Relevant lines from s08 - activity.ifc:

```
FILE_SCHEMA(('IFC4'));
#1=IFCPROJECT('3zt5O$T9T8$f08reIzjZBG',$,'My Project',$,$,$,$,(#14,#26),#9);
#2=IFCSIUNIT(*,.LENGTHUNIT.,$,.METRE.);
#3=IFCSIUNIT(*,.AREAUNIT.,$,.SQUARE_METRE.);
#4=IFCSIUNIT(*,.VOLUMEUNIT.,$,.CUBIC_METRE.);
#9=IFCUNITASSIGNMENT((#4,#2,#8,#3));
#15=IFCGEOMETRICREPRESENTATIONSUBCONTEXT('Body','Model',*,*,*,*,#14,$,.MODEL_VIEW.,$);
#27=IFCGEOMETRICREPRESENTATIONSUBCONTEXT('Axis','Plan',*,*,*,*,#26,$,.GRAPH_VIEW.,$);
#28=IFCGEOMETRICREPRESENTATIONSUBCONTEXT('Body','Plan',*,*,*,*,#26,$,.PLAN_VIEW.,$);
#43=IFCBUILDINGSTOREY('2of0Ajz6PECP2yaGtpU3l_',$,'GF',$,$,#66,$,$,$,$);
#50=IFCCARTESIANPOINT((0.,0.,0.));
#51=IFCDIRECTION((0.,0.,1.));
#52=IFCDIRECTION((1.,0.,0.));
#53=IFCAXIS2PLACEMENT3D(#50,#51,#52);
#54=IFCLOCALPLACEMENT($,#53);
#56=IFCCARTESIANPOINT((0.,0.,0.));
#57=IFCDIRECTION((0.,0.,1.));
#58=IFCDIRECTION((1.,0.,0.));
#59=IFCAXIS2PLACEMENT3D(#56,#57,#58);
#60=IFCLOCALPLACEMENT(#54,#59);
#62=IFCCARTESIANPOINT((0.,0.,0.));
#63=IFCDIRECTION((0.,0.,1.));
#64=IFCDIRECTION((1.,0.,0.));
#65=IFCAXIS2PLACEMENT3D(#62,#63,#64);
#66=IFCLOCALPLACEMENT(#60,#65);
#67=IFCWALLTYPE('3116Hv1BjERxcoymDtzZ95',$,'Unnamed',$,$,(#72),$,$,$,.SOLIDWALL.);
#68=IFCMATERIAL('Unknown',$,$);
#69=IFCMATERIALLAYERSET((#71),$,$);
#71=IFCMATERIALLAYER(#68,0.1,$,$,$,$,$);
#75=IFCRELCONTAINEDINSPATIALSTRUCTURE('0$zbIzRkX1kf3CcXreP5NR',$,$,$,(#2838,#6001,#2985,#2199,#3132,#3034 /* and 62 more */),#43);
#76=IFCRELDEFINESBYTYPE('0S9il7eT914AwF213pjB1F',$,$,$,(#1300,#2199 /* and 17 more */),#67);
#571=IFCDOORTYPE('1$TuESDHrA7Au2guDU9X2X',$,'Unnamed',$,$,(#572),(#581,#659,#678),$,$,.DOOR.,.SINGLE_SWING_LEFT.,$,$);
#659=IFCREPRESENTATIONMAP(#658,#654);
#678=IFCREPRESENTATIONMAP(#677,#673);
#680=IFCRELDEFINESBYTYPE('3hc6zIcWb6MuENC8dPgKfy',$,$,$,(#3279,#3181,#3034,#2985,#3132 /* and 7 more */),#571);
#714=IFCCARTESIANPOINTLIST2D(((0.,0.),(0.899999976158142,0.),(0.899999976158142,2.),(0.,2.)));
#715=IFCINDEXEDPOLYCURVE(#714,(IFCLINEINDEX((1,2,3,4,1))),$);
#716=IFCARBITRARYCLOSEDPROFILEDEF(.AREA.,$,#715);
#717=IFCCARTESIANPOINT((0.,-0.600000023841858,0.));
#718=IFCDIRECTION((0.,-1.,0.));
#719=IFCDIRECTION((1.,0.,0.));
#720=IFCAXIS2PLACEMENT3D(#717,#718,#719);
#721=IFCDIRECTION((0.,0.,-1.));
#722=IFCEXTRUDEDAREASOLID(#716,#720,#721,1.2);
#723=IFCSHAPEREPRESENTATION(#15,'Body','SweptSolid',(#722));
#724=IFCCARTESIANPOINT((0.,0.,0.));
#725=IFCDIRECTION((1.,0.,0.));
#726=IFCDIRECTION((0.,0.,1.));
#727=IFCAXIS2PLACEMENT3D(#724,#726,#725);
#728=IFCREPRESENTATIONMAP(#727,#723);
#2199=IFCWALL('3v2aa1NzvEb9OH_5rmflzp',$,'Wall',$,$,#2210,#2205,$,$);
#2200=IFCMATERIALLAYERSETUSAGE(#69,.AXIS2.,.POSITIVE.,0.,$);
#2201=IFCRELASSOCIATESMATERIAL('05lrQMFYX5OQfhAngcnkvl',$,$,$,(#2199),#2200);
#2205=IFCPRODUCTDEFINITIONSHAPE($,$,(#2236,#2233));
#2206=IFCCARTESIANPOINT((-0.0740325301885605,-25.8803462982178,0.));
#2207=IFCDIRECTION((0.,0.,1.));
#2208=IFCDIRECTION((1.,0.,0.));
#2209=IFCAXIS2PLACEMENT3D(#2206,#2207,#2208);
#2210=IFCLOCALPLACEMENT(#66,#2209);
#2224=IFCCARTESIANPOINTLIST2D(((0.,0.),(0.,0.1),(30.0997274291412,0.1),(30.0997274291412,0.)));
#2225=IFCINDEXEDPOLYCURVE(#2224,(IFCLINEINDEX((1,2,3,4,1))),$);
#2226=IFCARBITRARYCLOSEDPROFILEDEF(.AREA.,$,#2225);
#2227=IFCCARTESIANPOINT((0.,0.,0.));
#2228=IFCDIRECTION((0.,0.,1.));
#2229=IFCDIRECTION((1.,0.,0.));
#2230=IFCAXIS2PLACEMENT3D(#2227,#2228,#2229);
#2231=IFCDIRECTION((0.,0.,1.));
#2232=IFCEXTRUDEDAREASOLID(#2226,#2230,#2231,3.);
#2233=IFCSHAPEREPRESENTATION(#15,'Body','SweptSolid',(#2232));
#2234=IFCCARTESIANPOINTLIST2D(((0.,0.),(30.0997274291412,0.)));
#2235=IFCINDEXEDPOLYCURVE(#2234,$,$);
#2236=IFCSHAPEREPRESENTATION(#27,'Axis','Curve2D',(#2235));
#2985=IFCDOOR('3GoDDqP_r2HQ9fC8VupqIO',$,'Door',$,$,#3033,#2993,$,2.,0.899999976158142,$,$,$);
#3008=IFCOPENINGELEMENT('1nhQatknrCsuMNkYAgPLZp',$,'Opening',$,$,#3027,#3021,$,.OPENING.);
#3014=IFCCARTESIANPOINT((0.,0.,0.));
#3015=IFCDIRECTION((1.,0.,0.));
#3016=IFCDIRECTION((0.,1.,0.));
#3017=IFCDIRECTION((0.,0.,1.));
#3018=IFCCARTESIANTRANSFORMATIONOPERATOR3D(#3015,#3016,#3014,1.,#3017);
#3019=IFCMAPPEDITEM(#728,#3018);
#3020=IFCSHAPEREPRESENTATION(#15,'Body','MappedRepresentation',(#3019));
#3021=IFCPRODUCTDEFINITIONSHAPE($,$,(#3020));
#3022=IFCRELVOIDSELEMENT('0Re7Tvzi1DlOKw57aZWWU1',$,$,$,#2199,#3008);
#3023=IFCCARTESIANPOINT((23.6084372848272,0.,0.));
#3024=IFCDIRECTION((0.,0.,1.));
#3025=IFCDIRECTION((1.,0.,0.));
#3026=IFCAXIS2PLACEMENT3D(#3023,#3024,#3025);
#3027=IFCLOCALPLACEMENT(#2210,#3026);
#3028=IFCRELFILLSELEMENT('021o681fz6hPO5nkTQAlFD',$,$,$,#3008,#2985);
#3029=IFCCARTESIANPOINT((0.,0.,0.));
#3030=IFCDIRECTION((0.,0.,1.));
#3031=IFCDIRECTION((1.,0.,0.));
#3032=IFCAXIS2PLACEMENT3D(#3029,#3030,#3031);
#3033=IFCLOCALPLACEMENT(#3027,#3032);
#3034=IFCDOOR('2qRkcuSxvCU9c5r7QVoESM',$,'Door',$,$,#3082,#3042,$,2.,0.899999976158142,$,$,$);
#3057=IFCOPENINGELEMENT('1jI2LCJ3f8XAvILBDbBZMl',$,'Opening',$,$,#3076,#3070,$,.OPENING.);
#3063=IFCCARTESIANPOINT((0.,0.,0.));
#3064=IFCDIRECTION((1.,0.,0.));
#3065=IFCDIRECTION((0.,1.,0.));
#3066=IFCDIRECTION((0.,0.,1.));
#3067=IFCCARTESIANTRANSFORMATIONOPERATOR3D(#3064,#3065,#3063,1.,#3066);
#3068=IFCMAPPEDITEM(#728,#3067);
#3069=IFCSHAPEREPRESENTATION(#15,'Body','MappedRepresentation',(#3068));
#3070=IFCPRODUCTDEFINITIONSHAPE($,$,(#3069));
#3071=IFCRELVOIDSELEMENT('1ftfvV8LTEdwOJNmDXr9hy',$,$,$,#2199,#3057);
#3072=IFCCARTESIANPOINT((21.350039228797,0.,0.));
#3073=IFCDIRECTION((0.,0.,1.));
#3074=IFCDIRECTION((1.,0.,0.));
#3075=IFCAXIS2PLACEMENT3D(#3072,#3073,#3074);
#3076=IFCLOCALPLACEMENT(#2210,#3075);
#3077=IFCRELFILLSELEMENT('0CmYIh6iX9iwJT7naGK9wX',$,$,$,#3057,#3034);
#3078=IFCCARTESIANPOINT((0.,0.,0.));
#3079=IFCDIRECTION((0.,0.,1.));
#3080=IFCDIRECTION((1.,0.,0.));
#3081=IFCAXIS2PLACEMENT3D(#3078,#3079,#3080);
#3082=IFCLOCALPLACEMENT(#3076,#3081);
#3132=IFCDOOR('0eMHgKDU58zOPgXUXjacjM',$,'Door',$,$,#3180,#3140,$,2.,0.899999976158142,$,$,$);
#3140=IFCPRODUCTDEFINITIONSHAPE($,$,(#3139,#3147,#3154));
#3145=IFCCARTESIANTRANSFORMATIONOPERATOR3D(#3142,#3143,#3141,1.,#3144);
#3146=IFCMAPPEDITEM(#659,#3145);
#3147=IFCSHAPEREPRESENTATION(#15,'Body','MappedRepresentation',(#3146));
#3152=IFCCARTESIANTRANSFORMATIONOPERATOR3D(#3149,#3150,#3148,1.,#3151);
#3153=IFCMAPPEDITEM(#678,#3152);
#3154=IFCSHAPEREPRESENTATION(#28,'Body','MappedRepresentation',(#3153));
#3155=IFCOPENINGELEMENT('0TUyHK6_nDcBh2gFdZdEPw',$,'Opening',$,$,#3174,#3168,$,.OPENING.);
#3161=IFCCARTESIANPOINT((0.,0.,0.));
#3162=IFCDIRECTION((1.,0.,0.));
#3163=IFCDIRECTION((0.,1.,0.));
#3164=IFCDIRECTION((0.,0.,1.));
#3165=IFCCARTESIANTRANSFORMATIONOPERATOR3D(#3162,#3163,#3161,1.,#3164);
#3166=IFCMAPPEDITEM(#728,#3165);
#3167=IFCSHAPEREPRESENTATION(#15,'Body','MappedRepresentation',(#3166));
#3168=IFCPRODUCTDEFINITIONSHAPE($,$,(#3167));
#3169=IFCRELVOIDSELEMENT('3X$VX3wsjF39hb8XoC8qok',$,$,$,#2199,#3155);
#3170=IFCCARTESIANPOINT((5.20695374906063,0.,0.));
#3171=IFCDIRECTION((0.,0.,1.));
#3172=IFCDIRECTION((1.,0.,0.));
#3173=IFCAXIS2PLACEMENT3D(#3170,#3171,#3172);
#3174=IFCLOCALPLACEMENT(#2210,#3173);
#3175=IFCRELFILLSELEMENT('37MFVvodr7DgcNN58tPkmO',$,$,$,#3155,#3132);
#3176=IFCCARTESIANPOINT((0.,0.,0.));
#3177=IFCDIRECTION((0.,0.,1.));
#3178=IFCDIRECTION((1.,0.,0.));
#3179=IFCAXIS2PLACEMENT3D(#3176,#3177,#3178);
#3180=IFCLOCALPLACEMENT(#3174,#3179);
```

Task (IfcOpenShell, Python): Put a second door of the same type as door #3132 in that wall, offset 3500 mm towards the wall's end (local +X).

```python
import ifcopenshell
import ifcopenshell.api.feature
import ifcopenshell.api.geometry
import ifcopenshell.api.root
import ifcopenshell.geom
import ifcopenshell.util.element
import ifcopenshell.util.placement
import ifcopenshell.util.shape
import ifcopenshell.util.unit

model = ifcopenshell.open("s08 - activity.ifc")
unit_scale = ifcopenshell.util.unit.calculate_unit_scale(model)
settings = ifcopenshell.geom.settings()


def volume(element):
    """Net volume in cubic metres, openings subtracted."""
    shape = ifcopenshell.geom.create_shape(settings, element)
    return ifcopenshell.util.shape.get_volume(shape.geometry)


door = model.by_guid("0eMHgKDU58zOPgXUXjacjM")
opening = door.FillsVoids[0].RelatingOpeningElement
wall = opening.VoidsElements[0].RelatingBuildingElement
before = volume(wall)
shift = ifcopenshell.util.placement.get_local_placement(wall.ObjectPlacement)[:3, 0] * 3.5 / unit_scale

# copy_class copies the void relationship, type, container and properties, but no geometry.
new_opening = ifcopenshell.api.root.copy_class(model, product=opening)
new_opening.Representation = ifcopenshell.util.element.copy_deep(
    model, opening.Representation, exclude=["IfcGeometricRepresentationContext", "IfcRepresentationMap"]
)
new_door = ifcopenshell.api.root.copy_class(model, product=door)
new_door.Representation = ifcopenshell.util.element.copy_deep(
    model, door.Representation, exclude=["IfcGeometricRepresentationContext", "IfcRepresentationMap"]
)
ifcopenshell.api.feature.add_filling(model, opening=new_opening, element=new_door)

for old, new in ((opening, new_opening), (door, new_door)):
    matrix = ifcopenshell.util.placement.get_local_placement(old.ObjectPlacement)
    matrix[:3, 3] += shift
    ifcopenshell.api.geometry.edit_object_placement(model, product=new, matrix=matrix, is_si=False)

after = volume(wall)

print(f"wall volume {before:.3f} -> {after:.3f} m3")

model.write("s08 - activity_edited.ifc")
```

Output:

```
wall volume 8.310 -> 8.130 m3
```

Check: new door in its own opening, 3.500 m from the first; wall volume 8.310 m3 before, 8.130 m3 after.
